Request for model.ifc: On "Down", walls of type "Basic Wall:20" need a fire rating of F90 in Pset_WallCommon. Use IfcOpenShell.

First a look at what the model holds.

```python
import ifcopenshell
import ifcopenshell.util.element

model = ifcopenshell.open("model.ifc")
print(model.schema)
storey = next(s for s in model.by_type("IfcBuildingStorey") if s.Name == "Down")
walls = [e for e in ifcopenshell.util.element.get_decomposition(storey) if e.is_a("IfcWall")]
seen = {}
for e in walls:
    element_type = ifcopenshell.util.element.get_type(e)
    key = (element_type.Name if element_type != e and element_type else None, ifcopenshell.util.element.get_pset(e, "Pset_WallCommon", "FireRating"))
    seen[key] = seen.get(key, 0) + 1
for (name, value), count in sorted(seen.items(), key=str):
    print(count, "x", name, "|", value)
```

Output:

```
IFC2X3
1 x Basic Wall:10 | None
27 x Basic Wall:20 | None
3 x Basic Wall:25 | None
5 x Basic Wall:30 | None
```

```python
import ifcopenshell
import ifcopenshell.api.pset
import ifcopenshell.util.element

model = ifcopenshell.open("model.ifc")

storey = next(s for s in model.by_type("IfcBuildingStorey") if s.Name == "Down")
walls = [e for e in ifcopenshell.util.element.get_decomposition(storey) if e.is_a("IfcWall")]

count = 0
for e in walls:
    element_type = ifcopenshell.util.element.get_type(e)
    if element_type in (None, e) or element_type.Name != "Basic Wall:20":
        continue
    # add_pset returns the element's existing set when there is one.
    pset = ifcopenshell.api.pset.add_pset(model, product=e, name="Pset_WallCommon")
    ifcopenshell.api.pset.edit_pset(model, pset=pset, properties={"FireRating": "F90"})
    count += 1

print(count, "walls updated")

model.write("model_updated.ifc")
```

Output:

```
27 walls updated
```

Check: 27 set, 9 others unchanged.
